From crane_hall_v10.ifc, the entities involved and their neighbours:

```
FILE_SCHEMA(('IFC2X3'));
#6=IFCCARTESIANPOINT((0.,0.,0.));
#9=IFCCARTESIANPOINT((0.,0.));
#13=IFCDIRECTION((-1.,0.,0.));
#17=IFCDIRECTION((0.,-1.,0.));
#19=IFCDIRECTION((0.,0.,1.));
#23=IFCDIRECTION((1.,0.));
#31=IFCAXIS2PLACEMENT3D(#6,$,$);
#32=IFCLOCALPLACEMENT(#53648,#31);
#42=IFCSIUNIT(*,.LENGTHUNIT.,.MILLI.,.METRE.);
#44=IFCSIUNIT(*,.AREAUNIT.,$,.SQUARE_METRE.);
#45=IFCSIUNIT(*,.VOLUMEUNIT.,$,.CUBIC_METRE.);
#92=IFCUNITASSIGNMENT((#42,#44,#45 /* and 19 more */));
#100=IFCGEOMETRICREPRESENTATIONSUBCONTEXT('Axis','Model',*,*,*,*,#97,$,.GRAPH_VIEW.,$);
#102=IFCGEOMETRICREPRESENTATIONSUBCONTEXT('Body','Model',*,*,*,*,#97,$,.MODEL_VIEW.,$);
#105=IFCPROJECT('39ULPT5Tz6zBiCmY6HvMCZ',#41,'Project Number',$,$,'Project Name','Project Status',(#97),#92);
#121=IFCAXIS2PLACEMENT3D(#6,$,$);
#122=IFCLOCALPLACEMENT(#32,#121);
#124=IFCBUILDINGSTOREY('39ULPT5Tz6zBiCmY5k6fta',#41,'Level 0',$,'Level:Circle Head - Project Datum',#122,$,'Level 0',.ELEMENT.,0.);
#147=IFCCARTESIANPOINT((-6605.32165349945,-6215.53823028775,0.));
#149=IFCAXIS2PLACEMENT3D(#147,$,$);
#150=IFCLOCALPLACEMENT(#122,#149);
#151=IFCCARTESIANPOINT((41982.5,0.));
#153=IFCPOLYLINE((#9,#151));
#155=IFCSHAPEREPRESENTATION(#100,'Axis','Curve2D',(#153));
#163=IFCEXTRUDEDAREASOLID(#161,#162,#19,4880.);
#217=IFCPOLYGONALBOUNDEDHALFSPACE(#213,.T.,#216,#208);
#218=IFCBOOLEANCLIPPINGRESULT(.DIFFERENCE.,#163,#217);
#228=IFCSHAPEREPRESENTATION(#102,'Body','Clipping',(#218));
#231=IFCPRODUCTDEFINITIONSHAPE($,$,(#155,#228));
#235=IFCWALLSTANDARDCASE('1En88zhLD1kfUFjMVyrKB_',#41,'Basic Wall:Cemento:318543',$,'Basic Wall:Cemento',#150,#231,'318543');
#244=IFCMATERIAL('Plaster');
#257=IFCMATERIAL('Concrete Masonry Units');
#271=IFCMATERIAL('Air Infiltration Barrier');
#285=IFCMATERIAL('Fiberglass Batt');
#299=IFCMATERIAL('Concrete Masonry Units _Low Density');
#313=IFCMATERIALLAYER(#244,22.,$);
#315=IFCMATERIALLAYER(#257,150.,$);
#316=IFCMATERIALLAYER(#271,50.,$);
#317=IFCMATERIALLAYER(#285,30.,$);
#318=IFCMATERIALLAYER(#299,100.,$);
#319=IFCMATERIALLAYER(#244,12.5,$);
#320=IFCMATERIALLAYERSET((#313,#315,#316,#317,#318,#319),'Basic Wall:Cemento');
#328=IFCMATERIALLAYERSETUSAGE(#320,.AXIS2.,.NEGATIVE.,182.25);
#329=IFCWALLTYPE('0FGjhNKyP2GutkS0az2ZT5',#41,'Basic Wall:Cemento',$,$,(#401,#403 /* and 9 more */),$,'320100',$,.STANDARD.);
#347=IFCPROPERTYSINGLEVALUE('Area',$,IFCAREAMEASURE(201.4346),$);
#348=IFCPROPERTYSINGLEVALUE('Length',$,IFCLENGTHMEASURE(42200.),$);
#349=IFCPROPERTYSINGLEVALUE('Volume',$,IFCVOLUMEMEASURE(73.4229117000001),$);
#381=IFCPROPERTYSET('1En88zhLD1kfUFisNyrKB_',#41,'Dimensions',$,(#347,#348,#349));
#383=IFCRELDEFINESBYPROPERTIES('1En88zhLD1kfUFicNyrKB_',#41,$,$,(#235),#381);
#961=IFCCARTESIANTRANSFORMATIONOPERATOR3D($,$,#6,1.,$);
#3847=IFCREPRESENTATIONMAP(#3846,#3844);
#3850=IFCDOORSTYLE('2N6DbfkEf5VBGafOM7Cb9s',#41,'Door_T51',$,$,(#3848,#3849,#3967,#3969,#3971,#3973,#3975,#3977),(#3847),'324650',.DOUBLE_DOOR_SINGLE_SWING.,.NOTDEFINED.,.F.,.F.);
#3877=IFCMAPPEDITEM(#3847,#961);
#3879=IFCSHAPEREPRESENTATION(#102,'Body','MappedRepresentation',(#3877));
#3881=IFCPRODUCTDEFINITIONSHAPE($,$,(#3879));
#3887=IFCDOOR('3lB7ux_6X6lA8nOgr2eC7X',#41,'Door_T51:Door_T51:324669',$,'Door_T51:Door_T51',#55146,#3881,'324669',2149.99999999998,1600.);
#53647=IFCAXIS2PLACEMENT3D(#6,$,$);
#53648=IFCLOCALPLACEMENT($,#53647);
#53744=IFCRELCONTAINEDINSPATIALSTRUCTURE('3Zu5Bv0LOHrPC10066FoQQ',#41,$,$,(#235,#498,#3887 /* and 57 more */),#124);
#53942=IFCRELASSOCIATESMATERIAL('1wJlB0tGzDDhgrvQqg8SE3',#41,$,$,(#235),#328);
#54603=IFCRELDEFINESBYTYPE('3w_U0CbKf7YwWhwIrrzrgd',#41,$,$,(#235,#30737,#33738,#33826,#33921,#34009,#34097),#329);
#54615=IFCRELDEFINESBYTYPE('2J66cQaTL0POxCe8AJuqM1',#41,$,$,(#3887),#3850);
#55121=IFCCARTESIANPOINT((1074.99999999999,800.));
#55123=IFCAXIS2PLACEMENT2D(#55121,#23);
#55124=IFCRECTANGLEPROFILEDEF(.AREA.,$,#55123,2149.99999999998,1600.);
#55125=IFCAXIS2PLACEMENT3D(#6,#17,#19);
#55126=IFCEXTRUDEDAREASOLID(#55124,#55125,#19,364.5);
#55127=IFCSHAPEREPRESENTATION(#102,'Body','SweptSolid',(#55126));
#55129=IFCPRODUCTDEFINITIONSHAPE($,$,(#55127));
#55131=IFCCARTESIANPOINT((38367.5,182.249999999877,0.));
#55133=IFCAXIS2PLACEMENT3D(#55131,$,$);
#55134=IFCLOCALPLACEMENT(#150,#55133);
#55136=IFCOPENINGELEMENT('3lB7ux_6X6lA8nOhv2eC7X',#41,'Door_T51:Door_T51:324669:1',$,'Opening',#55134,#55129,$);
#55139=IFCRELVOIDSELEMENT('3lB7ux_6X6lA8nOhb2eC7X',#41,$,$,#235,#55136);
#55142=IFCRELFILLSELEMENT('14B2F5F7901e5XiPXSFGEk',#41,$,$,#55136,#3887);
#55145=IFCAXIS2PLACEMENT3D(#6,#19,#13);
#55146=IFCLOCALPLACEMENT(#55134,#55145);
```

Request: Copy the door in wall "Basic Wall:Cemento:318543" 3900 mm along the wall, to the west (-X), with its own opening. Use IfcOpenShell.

```python
import ifcopenshell
import ifcopenshell.api.feature
import ifcopenshell.api.geometry
import ifcopenshell.api.pset
import ifcopenshell.api.root
import ifcopenshell.geom
import ifcopenshell.util.element
import ifcopenshell.util.placement
import ifcopenshell.util.shape
import ifcopenshell.util.unit

model = ifcopenshell.open("crane_hall_v10.ifc")
area_scale = ifcopenshell.util.unit.calculate_unit_scale(model, "AREAUNIT")
volume_scale = ifcopenshell.util.unit.calculate_unit_scale(model, "VOLUMEUNIT")
settings = ifcopenshell.geom.settings()


def volume(element):
    """Net volume in cubic metres, openings subtracted."""
    shape = ifcopenshell.geom.create_shape(settings, element)
    return ifcopenshell.util.shape.get_volume(shape.geometry)


def reuse_history(source, copy):
    """copy_class also copies each property set's owner history, people and application; keep the originals."""
    for rel in copy.IsDefinedBy:
        if rel.is_a("IfcRelDefinesByProperties") and (history := rel.RelatingPropertyDefinition.OwnerHistory):
            rel.RelatingPropertyDefinition.OwnerHistory = source.OwnerHistory
            ifcopenshell.util.element.remove_deep2(model, history)


door = model.by_guid("3lB7ux_6X6lA8nOgr2eC7X")
opening = door.FillsVoids[0].RelatingOpeningElement
wall = opening.VoidsElements[0].RelatingBuildingElement
before = volume(wall)
shift = ifcopenshell.util.placement.get_local_placement(wall.ObjectPlacement)[:3, 0] * -3900.0

# copy_class copies the void relationship, type, container and properties, but no geometry.
new_opening = ifcopenshell.api.root.copy_class(model, product=opening)
new_opening.Representation = ifcopenshell.util.element.copy_deep(
    model, opening.Representation, exclude=["IfcGeometricRepresentationContext", "IfcRepresentationMap"]
)
new_opening.Name = "Door_T51:Door_T51"
new_door = ifcopenshell.api.root.copy_class(model, product=door)
new_door.Representation = ifcopenshell.util.element.copy_deep(
    model, door.Representation, exclude=["IfcGeometricRepresentationContext", "IfcRepresentationMap"]
)
new_door.Name = "Door_T51:Door_T51"
new_door.Tag = None
reuse_history(door, new_door)
fills = ifcopenshell.api.feature.add_filling(model, opening=new_opening, element=new_door)
fills.OwnerHistory = new_door.OwnerHistory  # required in IFC2X3

for old, new in ((opening, new_opening), (door, new_door)):
    matrix = ifcopenshell.util.placement.get_local_placement(old.ObjectPlacement)
    matrix[:3, 3] += shift
    ifcopenshell.api.geometry.edit_object_placement(model, product=new, matrix=matrix, is_si=False)

after = volume(wall)
thickness = 0.3645  # wall thickness in metres

# Update the wall's stored quantities.
pset = model.by_id(ifcopenshell.util.element.get_pset(wall, "Dimensions", should_inherit=False)["id"])
ifcopenshell.api.pset.edit_pset(model, pset=pset, properties={
    "Area": model.create_entity("IfcAreaMeasure", after / thickness / area_scale),
    "Volume": model.create_entity("IfcVolumeMeasure", after / volume_scale),
})

print(f"wall volume {before:.3f} -> {after:.3f} m3")

model.write("crane_hall_v10_edited.ifc")
```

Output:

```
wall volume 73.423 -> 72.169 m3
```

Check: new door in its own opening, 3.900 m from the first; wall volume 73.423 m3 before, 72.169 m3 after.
